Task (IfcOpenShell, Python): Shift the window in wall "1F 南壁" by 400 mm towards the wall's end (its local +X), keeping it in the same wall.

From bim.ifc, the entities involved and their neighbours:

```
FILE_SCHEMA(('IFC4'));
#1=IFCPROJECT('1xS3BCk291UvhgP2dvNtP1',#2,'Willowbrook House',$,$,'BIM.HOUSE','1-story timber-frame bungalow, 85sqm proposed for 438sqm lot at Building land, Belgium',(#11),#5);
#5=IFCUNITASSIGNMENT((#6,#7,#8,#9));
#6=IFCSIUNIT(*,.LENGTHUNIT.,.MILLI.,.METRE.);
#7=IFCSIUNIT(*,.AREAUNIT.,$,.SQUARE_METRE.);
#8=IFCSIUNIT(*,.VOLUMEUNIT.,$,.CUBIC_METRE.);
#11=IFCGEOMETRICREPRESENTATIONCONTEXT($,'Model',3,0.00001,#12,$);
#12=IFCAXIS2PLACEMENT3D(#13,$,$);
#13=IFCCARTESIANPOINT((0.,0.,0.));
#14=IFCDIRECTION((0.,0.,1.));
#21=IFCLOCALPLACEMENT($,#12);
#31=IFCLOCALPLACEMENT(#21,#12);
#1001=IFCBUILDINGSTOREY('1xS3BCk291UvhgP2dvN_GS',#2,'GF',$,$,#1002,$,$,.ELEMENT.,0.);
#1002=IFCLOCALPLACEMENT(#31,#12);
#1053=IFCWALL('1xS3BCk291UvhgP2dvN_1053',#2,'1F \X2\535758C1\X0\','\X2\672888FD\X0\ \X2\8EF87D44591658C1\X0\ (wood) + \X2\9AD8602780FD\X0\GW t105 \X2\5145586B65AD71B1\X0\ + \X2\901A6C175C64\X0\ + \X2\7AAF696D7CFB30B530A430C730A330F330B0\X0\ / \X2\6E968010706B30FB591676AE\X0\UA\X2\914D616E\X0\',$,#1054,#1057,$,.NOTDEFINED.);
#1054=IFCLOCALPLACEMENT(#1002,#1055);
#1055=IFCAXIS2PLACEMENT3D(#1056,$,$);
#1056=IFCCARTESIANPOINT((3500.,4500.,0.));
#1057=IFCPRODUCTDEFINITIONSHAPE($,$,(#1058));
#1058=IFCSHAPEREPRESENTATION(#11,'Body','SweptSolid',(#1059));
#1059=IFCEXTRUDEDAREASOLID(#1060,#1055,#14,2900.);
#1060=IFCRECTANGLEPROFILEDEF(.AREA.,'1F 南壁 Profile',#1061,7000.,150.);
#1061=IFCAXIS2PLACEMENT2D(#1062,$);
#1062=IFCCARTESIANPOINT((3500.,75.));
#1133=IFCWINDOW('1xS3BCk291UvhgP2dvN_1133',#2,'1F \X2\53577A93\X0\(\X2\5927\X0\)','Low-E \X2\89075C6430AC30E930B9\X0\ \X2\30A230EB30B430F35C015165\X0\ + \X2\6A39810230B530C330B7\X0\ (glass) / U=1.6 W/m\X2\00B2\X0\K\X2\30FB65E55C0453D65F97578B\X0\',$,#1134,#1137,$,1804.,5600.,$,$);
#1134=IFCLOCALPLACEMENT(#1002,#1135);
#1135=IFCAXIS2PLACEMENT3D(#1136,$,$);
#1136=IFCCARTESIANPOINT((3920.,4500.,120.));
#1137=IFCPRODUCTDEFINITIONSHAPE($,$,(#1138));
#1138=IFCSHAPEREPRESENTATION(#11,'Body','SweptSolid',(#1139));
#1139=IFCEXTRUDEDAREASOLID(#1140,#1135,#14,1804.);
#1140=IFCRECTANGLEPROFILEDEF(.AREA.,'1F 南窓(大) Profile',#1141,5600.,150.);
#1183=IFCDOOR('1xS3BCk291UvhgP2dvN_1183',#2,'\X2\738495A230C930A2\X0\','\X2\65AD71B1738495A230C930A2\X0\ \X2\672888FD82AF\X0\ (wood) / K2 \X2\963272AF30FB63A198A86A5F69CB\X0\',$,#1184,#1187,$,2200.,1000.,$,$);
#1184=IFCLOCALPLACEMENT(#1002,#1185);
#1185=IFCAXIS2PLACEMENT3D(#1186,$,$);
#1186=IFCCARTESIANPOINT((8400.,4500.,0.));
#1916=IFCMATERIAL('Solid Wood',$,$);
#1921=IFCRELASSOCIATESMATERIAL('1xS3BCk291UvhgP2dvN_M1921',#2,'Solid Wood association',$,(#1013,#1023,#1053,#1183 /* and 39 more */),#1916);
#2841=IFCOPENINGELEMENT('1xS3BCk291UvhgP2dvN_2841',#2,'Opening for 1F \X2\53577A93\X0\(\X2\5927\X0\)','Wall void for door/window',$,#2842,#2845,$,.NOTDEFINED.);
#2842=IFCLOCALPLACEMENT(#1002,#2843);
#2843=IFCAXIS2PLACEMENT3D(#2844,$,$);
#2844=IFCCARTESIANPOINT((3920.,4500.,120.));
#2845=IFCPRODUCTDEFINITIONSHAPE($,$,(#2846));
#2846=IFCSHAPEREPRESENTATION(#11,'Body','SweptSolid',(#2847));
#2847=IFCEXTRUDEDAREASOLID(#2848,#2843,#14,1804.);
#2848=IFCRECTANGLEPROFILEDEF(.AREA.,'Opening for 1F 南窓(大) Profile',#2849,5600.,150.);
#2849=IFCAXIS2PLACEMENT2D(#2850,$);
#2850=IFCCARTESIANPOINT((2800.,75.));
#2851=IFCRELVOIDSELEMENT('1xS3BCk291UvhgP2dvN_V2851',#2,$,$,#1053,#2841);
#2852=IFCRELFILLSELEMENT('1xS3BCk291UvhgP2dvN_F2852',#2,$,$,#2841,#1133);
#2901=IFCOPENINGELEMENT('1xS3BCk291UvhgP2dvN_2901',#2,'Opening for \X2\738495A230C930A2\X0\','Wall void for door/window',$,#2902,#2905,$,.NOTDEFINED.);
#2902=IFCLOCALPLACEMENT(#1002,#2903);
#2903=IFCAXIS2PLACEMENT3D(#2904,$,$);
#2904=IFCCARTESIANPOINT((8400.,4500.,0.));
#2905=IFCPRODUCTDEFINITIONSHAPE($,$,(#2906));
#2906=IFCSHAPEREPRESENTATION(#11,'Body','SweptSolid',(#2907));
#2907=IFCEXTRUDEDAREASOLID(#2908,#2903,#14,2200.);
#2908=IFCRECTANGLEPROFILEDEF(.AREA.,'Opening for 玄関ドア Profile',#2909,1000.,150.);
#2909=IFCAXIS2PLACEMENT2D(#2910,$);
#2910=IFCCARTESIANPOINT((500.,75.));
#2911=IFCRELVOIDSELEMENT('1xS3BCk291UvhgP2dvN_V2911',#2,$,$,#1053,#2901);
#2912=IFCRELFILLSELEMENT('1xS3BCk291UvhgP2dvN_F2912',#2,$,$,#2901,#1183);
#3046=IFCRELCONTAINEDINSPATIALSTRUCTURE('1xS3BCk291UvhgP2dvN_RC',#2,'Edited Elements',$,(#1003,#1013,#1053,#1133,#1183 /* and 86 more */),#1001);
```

```python
import ifcopenshell
import ifcopenshell.api.geometry
import ifcopenshell.util.placement

model = ifcopenshell.open("bim.ifc")

window = model.by_id(1133)
opening = window.FillsVoids[0].RelatingOpeningElement
wall = opening.VoidsElements[0].RelatingBuildingElement

wall_matrix = ifcopenshell.util.placement.get_local_placement(wall.ObjectPlacement)
shift = wall_matrix[:3, 0] * 400.0
before = ifcopenshell.util.placement.get_local_placement(window.ObjectPlacement)[:3, 3].copy()

# The window is not placed relative to its opening, so move both.
for product in (opening, window):
    matrix = ifcopenshell.util.placement.get_local_placement(product.ObjectPlacement)
    matrix[:3, 3] += shift
    ifcopenshell.api.geometry.edit_object_placement(model, product=product, matrix=matrix, is_si=False)

after = ifcopenshell.util.placement.get_local_placement(window.ObjectPlacement)[:3, 3]
print("window moved by", (after - before).round(3) + 0.0)

model.write("bim_edited.ifc")
```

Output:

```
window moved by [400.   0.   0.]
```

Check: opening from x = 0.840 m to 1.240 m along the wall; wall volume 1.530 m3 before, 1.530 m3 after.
